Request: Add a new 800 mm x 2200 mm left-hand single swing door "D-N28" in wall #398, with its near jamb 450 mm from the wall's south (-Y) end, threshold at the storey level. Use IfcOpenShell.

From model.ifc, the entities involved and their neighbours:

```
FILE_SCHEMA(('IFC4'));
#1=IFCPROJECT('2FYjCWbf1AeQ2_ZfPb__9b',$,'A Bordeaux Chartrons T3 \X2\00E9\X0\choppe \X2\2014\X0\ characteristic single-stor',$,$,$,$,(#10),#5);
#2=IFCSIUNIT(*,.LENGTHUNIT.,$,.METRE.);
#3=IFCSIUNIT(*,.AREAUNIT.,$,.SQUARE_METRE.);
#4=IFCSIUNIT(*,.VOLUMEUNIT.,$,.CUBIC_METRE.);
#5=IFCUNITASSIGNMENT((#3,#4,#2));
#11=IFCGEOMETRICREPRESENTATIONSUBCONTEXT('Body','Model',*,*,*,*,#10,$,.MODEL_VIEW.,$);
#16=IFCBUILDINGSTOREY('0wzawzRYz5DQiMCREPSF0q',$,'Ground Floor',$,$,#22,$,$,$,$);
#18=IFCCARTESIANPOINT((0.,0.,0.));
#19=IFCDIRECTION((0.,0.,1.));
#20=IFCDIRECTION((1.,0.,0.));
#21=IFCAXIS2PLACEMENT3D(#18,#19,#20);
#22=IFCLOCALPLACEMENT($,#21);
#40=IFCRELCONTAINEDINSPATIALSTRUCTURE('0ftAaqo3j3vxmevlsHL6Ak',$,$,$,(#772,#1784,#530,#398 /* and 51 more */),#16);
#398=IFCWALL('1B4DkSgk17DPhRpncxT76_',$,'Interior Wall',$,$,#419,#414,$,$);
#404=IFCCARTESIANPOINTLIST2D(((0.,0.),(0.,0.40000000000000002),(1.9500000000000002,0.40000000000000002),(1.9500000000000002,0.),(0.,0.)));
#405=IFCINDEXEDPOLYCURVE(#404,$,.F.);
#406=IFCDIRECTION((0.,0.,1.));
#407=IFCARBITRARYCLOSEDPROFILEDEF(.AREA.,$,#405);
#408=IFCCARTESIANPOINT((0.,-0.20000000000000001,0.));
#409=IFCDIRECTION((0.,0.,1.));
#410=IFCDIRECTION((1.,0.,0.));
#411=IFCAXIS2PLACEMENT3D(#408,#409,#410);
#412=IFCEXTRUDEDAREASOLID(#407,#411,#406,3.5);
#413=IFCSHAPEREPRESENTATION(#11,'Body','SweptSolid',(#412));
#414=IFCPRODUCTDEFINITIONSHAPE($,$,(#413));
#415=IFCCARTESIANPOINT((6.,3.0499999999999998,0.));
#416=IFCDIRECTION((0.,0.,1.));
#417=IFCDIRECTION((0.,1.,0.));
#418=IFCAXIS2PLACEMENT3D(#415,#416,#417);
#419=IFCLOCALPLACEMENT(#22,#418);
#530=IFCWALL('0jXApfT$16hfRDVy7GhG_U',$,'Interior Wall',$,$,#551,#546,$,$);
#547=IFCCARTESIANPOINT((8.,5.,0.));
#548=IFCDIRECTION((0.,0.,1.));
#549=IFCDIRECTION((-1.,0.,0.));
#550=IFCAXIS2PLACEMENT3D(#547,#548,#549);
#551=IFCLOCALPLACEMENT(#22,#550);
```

```python
import numpy as np
import ifcopenshell
import ifcopenshell.api.feature
import ifcopenshell.api.geometry
import ifcopenshell.api.root
import ifcopenshell.api.spatial
import ifcopenshell.geom
import ifcopenshell.util.element
import ifcopenshell.util.placement
import ifcopenshell.util.representation
import ifcopenshell.util.shape
import ifcopenshell.util.unit

model = ifcopenshell.open("model.ifc")
unit_scale = ifcopenshell.util.unit.calculate_unit_scale(model)
settings = ifcopenshell.geom.settings()


def volume(element):
    """Net volume in cubic metres, openings subtracted."""
    shape = ifcopenshell.geom.create_shape(settings, element)
    return ifcopenshell.util.shape.get_volume(shape.geometry)


wall = model.by_guid("1B4DkSgk17DPhRpncxT76_")
storey = ifcopenshell.util.element.get_container(wall, ifc_class="IfcBuildingStorey")
context = ifcopenshell.util.representation.get_context(model, "Model", "Body", "MODEL_VIEW")
before = volume(wall)

width, height, from_end, sill = 0.8, 2.2, 0.45, 0.0  # metres

# The wall runs along its own X axis, and the end named is its -X end.
wall_shape = ifcopenshell.geom.create_shape(settings, wall)
x, y, z = ifcopenshell.util.shape.get_vertices(wall_shape.geometry).T
start = x.min() + from_end
face, thickness = float(y.min()), float(y.max() - y.min())
wall_matrix = ifcopenshell.util.placement.get_local_placement(wall.ObjectPlacement)
level = ifcopenshell.util.placement.get_local_placement(storey.ObjectPlacement)[2, 3]


def in_wall(x, y):
    """Placement at x, y metres in the wall's axes, at sill height."""
    matrix = wall_matrix.copy()
    matrix[:, 3] = wall_matrix @ np.array([x / unit_scale, y / unit_scale, 0.0, 1.0])
    matrix[2, 3] = level + sill / unit_scale
    return matrix


# Opening: a box that overshoots both wall faces by 50 mm.
opening = ifcopenshell.api.root.create_entity(model, ifc_class="IfcOpeningElement", predefined_type="OPENING")
box = ifcopenshell.api.geometry.add_wall_representation(
    model, context=context, length=width, height=height, thickness=thickness + 0.1
)
ifcopenshell.api.geometry.assign_representation(model, product=opening, representation=box)
ifcopenshell.api.geometry.edit_object_placement(model, product=opening, matrix=in_wall(start, face - 0.05), is_si=False)
ifcopenshell.api.feature.add_feature(model, feature=opening, element=wall)

door = ifcopenshell.api.root.create_entity(model, ifc_class="IfcDoor", name="D-N28", predefined_type="DOOR")
door.OverallWidth, door.OverallHeight = width / unit_scale, height / unit_scale
door.OperationType = "SINGLE_SWING_LEFT"
body = ifcopenshell.api.geometry.add_door_representation(
    model,
    context=context,
    overall_width=door.OverallWidth,
    overall_height=door.OverallHeight,
    operation_type="SINGLE_SWING_LEFT",
    lining_properties={"LiningDepth": thickness / unit_scale, "ThresholdDepth": thickness / unit_scale},
)
ifcopenshell.api.geometry.assign_representation(model, product=door, representation=body)
ifcopenshell.api.spatial.assign_container(model, products=[door], relating_structure=storey)
ifcopenshell.api.feature.add_filling(model, opening=opening, element=door)

# The lining spans the wall, so the door starts at the wall face.
ifcopenshell.api.geometry.edit_object_placement(model, product=door, matrix=in_wall(start, face), is_si=False)

after = volume(wall)

print(f"wall volume {before:.3f} -> {after:.3f} m3")

model.write("model-out.ifc")
```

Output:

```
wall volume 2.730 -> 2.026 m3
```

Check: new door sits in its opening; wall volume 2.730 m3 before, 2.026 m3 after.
